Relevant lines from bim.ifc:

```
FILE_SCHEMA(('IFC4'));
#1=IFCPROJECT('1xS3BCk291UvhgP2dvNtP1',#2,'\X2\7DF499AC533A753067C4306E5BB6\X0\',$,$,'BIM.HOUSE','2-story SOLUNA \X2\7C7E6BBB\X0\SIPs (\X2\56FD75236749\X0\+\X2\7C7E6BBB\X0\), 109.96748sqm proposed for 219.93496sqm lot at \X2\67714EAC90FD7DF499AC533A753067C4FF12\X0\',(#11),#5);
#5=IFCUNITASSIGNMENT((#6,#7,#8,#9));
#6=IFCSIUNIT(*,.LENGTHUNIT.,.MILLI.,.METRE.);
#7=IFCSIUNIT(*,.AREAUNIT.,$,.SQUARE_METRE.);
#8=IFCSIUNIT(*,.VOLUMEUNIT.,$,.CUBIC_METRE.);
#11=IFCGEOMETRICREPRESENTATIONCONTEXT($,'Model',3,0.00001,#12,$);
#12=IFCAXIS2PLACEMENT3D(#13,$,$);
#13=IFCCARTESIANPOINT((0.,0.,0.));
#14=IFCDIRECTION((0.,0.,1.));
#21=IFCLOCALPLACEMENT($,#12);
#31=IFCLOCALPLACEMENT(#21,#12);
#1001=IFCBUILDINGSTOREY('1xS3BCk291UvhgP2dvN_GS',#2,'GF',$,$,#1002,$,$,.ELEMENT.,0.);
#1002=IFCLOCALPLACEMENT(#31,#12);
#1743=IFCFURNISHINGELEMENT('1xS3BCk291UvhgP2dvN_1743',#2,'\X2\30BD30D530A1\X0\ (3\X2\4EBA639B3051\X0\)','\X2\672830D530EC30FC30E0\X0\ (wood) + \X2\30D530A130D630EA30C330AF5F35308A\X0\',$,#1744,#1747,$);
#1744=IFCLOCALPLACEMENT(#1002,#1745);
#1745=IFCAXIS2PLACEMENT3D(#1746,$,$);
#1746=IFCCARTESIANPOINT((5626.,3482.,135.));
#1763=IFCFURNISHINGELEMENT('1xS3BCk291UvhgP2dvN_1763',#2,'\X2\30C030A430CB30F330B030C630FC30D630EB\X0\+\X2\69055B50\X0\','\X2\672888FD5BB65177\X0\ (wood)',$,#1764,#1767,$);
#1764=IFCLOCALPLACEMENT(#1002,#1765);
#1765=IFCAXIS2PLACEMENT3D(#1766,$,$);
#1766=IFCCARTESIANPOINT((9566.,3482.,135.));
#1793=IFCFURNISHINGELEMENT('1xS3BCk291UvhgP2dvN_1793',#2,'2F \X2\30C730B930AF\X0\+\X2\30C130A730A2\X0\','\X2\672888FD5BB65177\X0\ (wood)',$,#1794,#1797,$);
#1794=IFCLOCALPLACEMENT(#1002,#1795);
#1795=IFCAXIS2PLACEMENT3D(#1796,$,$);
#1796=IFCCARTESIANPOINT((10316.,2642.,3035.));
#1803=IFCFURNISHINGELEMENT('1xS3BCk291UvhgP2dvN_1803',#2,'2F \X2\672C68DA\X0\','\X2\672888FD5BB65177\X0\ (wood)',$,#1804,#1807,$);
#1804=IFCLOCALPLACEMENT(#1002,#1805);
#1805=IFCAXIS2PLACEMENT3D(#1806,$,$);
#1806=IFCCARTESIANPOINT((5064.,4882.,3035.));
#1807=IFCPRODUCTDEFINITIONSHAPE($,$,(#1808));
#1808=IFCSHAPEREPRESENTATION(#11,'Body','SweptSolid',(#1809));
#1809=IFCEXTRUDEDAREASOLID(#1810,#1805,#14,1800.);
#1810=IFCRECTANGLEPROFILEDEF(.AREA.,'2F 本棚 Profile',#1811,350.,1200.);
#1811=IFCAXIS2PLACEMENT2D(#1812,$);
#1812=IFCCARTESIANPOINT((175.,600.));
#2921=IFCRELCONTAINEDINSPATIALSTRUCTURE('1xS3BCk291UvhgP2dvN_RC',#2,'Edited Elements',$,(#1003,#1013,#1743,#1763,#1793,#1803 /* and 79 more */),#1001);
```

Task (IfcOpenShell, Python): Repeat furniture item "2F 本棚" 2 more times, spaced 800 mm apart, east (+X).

```python
import numpy as np
import ifcopenshell
import ifcopenshell.api.geometry
import ifcopenshell.api.root
import ifcopenshell.util.element
import ifcopenshell.util.placement

model = ifcopenshell.open("bim.ifc")


def reuse_history(source, copy):
    """copy_class also copies each property set's owner history, people and application; keep the originals."""
    for rel in copy.IsDefinedBy:
        if rel.is_a("IfcRelDefinesByProperties") and (history := rel.RelatingPropertyDefinition.OwnerHistory):
            rel.RelatingPropertyDefinition.OwnerHistory = source.OwnerHistory
            ifcopenshell.util.element.remove_deep2(model, history)


source = model.by_guid("1xS3BCk291UvhgP2dvN_1803")
base = ifcopenshell.util.placement.get_local_placement(source.ObjectPlacement)
step = np.array([1.0, 0.0, 0.0]) * 800.0

for i in range(1, 3):
    copy = ifcopenshell.api.root.copy_class(model, product=source)
    copy.Representation = ifcopenshell.util.element.copy_deep(
        model, source.Representation, exclude=["IfcGeometricRepresentationContext", "IfcRepresentationMap"]
    )
    reuse_history(source, copy)
    matrix = base.copy()
    matrix[:3, 3] += i * step
    print("added at", matrix[:3, 3].round(3) + 0.0)
    ifcopenshell.api.geometry.edit_object_placement(model, product=copy, matrix=matrix, is_si=False)

model.write("bim_edited.ifc")
```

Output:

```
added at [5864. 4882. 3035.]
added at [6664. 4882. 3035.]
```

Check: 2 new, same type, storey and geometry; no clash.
